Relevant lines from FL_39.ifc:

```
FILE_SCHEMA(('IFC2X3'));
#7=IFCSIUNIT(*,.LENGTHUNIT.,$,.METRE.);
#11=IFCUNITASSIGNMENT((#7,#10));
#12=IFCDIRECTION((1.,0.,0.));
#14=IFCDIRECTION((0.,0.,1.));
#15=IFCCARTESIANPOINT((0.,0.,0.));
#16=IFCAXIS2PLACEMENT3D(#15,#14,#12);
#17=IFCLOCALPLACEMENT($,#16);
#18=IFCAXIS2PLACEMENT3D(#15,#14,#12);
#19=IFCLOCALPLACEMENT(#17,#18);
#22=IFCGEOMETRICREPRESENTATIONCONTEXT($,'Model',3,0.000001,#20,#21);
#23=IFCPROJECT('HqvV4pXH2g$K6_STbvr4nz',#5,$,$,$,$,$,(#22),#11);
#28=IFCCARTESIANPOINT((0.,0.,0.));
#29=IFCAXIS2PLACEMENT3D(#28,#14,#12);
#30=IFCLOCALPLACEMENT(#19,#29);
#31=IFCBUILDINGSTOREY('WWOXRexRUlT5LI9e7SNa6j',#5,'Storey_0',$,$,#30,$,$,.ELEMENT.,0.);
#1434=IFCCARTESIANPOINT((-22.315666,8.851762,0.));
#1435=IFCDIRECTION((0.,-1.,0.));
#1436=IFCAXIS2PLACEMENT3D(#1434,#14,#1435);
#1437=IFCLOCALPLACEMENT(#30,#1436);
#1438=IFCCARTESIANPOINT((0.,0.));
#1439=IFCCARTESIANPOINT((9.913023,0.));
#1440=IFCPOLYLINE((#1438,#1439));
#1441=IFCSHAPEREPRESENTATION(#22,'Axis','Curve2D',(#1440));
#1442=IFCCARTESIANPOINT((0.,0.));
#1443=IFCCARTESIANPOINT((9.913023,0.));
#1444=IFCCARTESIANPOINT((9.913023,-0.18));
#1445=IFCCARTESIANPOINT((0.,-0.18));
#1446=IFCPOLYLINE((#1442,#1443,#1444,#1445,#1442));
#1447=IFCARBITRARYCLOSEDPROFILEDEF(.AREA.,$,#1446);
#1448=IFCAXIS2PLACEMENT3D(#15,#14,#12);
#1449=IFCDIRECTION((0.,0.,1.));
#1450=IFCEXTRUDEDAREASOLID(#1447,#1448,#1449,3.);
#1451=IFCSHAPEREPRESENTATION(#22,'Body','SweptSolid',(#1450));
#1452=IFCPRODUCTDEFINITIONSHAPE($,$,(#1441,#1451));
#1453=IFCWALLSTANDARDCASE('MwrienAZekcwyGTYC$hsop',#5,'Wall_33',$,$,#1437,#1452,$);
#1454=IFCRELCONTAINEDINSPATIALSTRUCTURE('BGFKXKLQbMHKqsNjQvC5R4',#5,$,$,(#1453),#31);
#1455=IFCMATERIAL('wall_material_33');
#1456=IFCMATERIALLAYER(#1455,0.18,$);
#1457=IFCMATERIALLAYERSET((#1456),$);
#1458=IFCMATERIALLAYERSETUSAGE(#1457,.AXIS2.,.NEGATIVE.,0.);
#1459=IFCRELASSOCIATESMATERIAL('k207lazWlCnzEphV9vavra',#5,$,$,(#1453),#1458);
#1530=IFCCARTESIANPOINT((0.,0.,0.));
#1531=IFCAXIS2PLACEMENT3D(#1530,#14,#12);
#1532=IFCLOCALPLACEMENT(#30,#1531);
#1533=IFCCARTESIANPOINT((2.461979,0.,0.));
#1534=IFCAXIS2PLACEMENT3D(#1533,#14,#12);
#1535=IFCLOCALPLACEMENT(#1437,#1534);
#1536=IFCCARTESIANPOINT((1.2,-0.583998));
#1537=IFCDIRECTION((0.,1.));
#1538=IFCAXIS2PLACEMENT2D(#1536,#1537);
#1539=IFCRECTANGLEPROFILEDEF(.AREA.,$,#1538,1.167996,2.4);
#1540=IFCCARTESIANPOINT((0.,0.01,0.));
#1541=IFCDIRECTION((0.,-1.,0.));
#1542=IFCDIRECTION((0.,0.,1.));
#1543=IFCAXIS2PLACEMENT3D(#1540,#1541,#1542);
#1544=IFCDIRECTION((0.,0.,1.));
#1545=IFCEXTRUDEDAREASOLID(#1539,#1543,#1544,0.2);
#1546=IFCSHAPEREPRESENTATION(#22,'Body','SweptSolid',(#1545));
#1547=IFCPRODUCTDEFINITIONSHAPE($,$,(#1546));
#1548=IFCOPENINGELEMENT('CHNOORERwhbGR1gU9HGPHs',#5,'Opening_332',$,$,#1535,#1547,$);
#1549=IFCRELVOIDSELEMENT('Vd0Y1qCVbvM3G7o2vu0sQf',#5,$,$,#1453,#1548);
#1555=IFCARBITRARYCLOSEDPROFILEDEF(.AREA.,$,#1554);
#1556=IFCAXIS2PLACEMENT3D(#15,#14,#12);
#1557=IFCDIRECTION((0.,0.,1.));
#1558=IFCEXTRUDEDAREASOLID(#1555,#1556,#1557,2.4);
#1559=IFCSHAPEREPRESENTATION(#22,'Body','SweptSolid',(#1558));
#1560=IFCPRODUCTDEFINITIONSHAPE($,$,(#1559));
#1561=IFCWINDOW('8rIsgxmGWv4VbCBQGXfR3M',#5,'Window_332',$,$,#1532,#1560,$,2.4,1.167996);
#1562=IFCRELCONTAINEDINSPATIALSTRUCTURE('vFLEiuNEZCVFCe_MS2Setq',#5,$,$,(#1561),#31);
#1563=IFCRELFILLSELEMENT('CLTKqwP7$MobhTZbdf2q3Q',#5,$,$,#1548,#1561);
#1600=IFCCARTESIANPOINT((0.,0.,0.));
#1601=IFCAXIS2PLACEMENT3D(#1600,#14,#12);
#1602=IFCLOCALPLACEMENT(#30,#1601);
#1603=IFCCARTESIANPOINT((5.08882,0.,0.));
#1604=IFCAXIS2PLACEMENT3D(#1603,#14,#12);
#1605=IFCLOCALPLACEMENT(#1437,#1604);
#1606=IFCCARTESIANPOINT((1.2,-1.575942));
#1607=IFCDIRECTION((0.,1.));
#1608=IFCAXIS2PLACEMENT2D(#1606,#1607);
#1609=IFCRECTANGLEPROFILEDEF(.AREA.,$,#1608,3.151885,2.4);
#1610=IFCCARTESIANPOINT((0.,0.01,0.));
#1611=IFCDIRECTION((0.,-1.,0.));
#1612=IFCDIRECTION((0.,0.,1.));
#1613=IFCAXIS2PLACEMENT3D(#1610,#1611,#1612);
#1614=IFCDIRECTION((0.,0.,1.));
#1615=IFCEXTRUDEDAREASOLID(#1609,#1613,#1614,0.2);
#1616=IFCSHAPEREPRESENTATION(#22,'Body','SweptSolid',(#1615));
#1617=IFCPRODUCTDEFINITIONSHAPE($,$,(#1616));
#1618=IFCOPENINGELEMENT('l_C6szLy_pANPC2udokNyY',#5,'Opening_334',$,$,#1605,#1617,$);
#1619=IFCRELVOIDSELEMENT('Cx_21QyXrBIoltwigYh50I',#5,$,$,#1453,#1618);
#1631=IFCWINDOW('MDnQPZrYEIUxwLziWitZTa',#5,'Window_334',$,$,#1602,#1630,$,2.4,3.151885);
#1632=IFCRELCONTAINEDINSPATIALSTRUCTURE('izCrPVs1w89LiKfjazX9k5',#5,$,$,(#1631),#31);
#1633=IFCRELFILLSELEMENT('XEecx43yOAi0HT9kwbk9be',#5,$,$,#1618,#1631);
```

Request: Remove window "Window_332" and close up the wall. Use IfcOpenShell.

```python
import ifcopenshell
import ifcopenshell.api.feature
import ifcopenshell.api.root
import ifcopenshell.geom
import ifcopenshell.util.shape

model = ifcopenshell.open("FL_39.ifc")
settings = ifcopenshell.geom.settings()


def volume(element):
    """Net volume in cubic metres, openings subtracted."""
    shape = ifcopenshell.geom.create_shape(settings, element)
    return ifcopenshell.util.shape.get_volume(shape.geometry)


window = model.by_guid("8rIsgxmGWv4VbCBQGXfR3M")
opening = window.FillsVoids[0].RelatingOpeningElement
wall = opening.VoidsElements[0].RelatingBuildingElement
before = volume(wall)

ifcopenshell.api.root.remove_product(model, product=window)
ifcopenshell.api.feature.remove_feature(model, feature=opening)

after = volume(wall)

print(f"wall volume {before:.3f} -> {after:.3f} m3")

model.write("FL_39_edited.ifc")
```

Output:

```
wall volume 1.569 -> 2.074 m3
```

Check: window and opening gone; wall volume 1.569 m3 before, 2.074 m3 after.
